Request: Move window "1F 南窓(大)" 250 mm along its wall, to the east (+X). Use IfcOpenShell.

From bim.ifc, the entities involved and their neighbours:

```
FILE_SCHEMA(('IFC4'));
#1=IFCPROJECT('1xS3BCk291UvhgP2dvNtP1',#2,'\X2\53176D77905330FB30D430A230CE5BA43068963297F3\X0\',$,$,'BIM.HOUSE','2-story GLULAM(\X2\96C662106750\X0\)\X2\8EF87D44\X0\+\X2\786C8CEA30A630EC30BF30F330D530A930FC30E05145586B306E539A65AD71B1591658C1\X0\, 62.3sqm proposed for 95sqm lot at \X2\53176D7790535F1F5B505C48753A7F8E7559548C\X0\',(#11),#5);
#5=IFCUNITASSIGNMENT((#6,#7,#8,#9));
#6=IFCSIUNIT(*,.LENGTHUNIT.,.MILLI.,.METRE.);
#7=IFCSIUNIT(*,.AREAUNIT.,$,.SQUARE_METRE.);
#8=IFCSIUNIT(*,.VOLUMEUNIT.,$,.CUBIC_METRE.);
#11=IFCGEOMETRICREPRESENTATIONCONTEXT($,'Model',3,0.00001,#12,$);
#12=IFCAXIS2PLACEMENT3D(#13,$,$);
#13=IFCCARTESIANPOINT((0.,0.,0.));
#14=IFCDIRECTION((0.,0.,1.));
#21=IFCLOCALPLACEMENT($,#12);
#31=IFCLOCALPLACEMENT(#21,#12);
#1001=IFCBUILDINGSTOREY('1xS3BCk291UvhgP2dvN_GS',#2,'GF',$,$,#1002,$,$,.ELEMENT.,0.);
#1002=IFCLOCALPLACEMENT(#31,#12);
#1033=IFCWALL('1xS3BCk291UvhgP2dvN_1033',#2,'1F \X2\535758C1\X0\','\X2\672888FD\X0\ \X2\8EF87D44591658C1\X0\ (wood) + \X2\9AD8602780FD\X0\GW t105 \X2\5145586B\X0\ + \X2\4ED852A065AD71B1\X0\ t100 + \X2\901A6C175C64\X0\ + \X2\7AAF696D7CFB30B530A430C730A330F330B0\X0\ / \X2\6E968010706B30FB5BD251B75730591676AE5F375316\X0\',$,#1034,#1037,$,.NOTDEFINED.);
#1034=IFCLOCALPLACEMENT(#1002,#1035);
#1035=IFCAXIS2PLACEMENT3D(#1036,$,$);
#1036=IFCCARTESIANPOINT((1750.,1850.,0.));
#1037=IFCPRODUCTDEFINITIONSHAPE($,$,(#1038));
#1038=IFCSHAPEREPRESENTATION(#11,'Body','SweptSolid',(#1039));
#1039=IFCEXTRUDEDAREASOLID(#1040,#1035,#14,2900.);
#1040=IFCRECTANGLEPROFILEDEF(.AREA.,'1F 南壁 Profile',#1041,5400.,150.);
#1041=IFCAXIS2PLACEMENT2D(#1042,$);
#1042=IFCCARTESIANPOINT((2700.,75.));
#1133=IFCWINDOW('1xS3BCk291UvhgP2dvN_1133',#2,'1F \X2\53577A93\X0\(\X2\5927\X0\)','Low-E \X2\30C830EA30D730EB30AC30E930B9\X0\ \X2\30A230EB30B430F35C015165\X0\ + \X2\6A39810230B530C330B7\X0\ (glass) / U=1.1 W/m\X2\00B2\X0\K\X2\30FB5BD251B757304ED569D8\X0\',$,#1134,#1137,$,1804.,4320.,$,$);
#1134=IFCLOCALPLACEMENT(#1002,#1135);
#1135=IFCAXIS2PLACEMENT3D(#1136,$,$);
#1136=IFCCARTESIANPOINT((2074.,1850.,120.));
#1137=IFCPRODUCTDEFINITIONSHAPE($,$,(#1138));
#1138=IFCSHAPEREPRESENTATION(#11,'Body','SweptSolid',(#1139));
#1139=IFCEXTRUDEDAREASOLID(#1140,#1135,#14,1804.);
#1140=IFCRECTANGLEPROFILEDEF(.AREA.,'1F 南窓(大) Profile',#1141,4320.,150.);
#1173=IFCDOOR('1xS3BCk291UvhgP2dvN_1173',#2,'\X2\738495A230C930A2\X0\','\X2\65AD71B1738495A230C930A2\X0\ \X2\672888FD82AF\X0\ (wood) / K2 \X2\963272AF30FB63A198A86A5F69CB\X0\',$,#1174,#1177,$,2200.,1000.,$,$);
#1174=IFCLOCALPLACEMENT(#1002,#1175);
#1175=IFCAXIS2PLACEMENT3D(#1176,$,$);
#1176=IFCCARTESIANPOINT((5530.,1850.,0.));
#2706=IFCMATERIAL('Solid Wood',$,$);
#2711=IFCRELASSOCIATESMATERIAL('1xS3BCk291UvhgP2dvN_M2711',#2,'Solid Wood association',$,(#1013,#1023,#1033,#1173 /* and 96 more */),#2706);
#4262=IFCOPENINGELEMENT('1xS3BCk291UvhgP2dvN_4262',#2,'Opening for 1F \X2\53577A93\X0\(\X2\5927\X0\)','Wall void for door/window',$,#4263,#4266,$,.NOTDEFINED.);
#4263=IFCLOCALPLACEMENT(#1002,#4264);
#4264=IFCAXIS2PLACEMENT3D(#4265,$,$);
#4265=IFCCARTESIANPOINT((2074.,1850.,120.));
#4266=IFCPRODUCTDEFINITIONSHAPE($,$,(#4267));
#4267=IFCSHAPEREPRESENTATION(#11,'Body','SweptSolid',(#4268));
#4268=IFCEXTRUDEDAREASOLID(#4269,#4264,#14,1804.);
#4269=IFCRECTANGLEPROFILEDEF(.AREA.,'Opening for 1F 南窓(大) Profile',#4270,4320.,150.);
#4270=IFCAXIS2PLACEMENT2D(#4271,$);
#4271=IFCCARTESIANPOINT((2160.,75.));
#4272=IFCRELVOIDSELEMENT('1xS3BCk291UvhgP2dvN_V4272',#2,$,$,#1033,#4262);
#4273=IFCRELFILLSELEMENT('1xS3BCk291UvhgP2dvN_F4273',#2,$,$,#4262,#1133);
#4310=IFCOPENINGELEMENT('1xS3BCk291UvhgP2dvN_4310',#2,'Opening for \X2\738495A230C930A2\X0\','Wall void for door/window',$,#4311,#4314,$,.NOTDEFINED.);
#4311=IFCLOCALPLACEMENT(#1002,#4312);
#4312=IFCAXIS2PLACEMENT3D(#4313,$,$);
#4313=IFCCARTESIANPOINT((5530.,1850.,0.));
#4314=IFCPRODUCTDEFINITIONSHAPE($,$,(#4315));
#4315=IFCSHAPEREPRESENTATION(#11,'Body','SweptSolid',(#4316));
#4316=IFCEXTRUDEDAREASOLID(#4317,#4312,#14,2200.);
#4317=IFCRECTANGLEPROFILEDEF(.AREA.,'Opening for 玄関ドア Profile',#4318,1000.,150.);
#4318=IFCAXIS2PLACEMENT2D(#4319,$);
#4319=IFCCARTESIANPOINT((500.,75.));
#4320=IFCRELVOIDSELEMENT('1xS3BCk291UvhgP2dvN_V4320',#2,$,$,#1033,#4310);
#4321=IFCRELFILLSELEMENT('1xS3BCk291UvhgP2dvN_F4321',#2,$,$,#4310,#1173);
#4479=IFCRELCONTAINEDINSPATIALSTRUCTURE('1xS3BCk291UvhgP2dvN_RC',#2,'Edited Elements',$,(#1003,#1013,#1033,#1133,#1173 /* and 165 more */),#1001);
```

```python
import ifcopenshell
import ifcopenshell.api.geometry
import ifcopenshell.util.placement
import ifcopenshell.util.unit

model = ifcopenshell.open("bim.ifc")
unit_scale = ifcopenshell.util.unit.calculate_unit_scale(model)

window = model.by_guid("1xS3BCk291UvhgP2dvN_1133")
opening = window.FillsVoids[0].RelatingOpeningElement
wall = opening.VoidsElements[0].RelatingBuildingElement

wall_matrix = ifcopenshell.util.placement.get_local_placement(wall.ObjectPlacement)
shift = wall_matrix[:3, 0] * 0.25 / unit_scale
before = ifcopenshell.util.placement.get_local_placement(window.ObjectPlacement)[:3, 3].copy()

# The window is not placed relative to its opening, so move both.
for product in (opening, window):
    matrix = ifcopenshell.util.placement.get_local_placement(product.ObjectPlacement)
    matrix[:3, 3] += shift
    ifcopenshell.api.geometry.edit_object_placement(model, product=product, matrix=matrix, is_si=False)

after = ifcopenshell.util.placement.get_local_placement(window.ObjectPlacement)[:3, 3]
print("window moved by", (after - before).round(3) + 0.0)

model.write("bim_edited.ifc")
```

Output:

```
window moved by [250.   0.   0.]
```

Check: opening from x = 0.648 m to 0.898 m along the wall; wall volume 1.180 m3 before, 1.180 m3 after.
